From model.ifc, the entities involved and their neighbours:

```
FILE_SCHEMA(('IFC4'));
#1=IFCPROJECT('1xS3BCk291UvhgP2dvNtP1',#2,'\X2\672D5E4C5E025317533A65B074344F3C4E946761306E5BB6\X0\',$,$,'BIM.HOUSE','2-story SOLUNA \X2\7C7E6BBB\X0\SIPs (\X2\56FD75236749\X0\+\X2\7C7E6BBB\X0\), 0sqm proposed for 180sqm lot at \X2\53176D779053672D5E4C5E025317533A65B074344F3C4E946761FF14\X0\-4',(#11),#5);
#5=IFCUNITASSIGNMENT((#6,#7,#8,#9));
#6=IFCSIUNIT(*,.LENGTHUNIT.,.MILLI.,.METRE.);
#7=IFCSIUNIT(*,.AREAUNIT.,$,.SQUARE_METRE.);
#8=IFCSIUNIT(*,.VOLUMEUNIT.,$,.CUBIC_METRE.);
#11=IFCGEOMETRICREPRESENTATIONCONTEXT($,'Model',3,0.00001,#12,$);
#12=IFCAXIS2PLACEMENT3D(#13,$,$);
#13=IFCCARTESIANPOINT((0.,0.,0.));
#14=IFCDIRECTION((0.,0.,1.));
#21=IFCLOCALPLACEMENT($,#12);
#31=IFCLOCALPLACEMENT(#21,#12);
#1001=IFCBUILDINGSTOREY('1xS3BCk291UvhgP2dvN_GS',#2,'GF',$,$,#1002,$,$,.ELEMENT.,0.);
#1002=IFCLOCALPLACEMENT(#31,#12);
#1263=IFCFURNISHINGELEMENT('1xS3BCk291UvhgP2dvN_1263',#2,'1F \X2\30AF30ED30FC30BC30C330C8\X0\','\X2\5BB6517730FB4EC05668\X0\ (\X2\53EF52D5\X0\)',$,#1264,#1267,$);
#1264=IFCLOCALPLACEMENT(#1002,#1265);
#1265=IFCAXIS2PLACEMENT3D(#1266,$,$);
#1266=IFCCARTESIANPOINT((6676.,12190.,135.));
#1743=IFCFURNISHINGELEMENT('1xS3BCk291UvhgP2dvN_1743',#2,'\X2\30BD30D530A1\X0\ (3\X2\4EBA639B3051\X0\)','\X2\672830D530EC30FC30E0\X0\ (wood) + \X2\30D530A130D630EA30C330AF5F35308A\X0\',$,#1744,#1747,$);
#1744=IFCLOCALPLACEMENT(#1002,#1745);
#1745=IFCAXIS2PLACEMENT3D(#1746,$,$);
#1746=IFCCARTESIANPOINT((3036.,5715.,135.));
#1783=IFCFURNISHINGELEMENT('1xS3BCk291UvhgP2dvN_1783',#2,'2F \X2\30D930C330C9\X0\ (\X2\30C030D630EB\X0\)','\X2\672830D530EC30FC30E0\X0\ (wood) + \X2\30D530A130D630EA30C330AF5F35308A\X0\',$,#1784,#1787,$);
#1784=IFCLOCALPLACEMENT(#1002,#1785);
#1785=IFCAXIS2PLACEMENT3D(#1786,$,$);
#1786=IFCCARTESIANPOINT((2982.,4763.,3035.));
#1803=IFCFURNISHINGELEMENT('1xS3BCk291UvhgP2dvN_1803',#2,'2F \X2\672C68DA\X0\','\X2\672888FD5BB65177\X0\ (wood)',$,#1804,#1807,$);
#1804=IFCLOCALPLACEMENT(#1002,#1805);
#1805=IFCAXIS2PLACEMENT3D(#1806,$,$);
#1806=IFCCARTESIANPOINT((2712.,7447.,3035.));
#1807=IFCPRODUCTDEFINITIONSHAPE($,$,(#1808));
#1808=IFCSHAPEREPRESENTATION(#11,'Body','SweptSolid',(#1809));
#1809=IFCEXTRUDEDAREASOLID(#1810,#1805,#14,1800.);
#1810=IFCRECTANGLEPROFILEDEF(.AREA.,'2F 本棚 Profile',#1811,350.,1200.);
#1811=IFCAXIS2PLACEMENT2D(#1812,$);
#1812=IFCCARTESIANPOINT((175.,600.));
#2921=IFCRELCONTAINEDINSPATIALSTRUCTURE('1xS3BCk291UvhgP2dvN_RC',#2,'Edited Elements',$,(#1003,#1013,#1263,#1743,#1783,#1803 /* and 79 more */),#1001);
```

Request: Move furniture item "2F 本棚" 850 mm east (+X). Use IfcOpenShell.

```python
import ifcopenshell
import ifcopenshell.api.geometry
import ifcopenshell.util.placement

model = ifcopenshell.open("model.ifc")

item = model.by_guid("1xS3BCk291UvhgP2dvN_1803")
matrix = ifcopenshell.util.placement.get_local_placement(item.ObjectPlacement)
matrix[0, 3] += 850.0
ifcopenshell.api.geometry.edit_object_placement(model, product=item, matrix=matrix, is_si=False)

print(ifcopenshell.util.placement.get_local_placement(item.ObjectPlacement).round(3) + 0.0)

model.write("model_v2.ifc")
```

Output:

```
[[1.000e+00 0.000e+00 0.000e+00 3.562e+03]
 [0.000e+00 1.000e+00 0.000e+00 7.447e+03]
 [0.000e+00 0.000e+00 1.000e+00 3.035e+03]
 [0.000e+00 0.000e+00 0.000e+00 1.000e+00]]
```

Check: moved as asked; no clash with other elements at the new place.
